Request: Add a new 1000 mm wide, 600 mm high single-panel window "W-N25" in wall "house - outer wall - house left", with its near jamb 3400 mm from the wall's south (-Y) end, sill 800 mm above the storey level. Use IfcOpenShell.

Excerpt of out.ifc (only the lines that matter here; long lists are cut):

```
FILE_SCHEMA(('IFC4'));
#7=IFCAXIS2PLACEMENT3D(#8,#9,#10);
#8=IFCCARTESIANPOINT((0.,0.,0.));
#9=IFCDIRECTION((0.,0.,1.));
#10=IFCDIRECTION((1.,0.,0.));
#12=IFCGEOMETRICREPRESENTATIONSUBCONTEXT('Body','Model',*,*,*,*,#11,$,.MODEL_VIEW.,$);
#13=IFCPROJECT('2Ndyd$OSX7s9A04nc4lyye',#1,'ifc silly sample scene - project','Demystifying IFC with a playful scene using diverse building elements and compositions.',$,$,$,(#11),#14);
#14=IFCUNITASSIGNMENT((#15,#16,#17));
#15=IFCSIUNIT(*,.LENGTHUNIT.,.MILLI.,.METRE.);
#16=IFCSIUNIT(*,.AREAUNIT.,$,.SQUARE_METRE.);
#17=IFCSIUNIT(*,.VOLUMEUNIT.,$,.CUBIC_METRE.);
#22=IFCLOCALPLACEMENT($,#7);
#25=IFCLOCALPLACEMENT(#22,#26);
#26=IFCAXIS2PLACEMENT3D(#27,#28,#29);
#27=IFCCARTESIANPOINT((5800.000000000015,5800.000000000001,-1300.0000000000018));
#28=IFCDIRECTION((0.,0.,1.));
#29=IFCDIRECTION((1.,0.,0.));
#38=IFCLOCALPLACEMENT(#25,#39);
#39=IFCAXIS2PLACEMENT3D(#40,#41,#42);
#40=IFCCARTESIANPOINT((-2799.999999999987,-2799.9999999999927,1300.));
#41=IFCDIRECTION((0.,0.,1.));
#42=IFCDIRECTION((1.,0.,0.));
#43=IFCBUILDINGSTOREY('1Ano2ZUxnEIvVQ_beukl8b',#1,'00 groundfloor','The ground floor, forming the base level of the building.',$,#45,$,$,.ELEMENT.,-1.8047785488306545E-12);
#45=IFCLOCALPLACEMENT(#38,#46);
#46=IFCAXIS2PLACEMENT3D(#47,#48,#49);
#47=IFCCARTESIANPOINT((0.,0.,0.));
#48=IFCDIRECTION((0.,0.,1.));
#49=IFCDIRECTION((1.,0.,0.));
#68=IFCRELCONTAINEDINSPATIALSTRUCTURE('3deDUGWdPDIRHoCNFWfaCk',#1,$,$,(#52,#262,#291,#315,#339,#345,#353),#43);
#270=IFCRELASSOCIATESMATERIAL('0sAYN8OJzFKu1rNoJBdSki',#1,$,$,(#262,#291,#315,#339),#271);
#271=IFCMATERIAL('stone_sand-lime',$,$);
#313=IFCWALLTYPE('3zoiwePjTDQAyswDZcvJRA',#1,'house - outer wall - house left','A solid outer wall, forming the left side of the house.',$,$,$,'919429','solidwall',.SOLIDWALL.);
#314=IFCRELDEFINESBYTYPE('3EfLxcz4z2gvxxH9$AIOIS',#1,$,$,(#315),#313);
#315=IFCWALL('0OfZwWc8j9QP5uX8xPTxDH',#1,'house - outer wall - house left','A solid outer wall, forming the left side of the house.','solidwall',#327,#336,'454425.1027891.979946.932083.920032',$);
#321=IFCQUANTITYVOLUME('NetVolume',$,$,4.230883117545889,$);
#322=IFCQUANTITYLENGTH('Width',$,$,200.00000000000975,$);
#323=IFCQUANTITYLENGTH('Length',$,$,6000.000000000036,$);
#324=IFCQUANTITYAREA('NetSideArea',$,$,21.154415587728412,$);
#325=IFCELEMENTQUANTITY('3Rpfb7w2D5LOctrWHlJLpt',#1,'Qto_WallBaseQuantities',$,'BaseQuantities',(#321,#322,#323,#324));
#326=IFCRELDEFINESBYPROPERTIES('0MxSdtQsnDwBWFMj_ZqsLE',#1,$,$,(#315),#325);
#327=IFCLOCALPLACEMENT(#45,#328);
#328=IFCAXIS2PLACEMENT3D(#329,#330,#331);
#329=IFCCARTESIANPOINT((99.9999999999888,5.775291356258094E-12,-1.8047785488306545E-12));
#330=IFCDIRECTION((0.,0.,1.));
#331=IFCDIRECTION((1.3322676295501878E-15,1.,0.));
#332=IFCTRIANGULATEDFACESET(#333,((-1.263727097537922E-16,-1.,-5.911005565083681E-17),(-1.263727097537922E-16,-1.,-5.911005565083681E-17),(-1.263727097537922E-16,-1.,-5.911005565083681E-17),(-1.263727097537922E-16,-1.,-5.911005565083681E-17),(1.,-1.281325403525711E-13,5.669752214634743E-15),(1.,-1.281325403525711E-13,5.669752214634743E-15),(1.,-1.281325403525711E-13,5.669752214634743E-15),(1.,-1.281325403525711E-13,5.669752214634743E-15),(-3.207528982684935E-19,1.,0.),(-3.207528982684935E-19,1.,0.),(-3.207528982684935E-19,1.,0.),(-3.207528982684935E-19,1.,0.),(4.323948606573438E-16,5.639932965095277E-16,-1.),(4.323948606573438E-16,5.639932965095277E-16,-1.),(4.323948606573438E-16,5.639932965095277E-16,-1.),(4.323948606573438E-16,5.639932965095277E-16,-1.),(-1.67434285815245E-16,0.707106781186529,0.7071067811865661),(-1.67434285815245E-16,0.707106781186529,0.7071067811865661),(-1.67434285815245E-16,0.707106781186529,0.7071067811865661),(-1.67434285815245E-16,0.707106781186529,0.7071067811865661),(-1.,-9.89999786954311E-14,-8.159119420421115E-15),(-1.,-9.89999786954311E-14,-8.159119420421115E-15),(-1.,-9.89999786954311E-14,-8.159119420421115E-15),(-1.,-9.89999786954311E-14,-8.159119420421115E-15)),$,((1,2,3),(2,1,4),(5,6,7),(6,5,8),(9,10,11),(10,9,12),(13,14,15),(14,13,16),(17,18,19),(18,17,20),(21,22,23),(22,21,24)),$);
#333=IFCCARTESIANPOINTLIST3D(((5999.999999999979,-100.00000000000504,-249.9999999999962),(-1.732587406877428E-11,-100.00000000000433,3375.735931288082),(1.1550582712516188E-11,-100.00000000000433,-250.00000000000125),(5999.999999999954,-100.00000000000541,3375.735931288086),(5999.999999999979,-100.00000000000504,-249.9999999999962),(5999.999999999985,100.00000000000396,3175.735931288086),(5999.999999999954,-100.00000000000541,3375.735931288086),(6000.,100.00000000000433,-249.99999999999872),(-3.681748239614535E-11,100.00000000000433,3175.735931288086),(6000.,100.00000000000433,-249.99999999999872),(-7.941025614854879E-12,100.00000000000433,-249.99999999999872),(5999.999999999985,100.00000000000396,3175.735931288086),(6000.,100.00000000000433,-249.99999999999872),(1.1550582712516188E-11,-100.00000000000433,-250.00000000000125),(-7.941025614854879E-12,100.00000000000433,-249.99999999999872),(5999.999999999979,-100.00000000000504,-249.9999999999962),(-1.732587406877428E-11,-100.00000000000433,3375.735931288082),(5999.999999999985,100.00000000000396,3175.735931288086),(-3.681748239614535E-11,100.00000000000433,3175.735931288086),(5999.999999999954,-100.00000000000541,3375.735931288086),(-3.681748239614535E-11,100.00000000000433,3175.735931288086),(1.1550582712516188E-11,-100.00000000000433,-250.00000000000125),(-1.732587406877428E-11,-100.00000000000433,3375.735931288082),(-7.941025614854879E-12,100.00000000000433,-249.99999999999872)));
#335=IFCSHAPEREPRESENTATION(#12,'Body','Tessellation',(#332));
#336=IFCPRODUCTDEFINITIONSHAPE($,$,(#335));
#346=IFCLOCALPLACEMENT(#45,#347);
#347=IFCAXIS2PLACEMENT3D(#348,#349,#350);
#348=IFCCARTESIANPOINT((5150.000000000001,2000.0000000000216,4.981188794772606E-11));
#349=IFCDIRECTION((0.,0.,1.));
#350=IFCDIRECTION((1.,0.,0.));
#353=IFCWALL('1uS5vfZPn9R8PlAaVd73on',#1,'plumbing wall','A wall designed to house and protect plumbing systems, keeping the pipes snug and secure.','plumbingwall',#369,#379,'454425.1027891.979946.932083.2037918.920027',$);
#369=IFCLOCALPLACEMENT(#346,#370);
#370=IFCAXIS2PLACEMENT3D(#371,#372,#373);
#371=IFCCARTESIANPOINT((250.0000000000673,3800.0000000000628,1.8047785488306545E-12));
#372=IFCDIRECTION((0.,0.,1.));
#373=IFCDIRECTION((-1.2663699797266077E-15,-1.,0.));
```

```python
import numpy as np
import ifcopenshell
import ifcopenshell.api.feature
import ifcopenshell.api.geometry
import ifcopenshell.api.pset
import ifcopenshell.api.root
import ifcopenshell.api.spatial
import ifcopenshell.geom
import ifcopenshell.util.element
import ifcopenshell.util.placement
import ifcopenshell.util.representation
import ifcopenshell.util.shape
import ifcopenshell.util.unit

model = ifcopenshell.open("out.ifc")
unit_scale = ifcopenshell.util.unit.calculate_unit_scale(model)
area_scale = ifcopenshell.util.unit.calculate_unit_scale(model, "AREAUNIT")
volume_scale = ifcopenshell.util.unit.calculate_unit_scale(model, "VOLUMEUNIT")
settings = ifcopenshell.geom.settings()


def volume(element):
    """Net volume in cubic metres, openings subtracted."""
    shape = ifcopenshell.geom.create_shape(settings, element)
    return ifcopenshell.util.shape.get_volume(shape.geometry)


wall = model.by_guid("0OfZwWc8j9QP5uX8xPTxDH")
storey = ifcopenshell.util.element.get_container(wall, ifc_class="IfcBuildingStorey")
context = ifcopenshell.util.representation.get_context(model, "Model", "Body", "MODEL_VIEW")
before = volume(wall)

width, height, from_end, sill = 1, 0.6, 3.4, 0.8  # metres

# The wall runs along its own X axis, and the end named is its -X end.
wall_shape = ifcopenshell.geom.create_shape(settings, wall)
x, y, z = ifcopenshell.util.shape.get_vertices(wall_shape.geometry).T
start = x.min() + from_end
face, thickness = float(y.min()), float(y.max() - y.min())
wall_matrix = ifcopenshell.util.placement.get_local_placement(wall.ObjectPlacement)
level = ifcopenshell.util.placement.get_local_placement(storey.ObjectPlacement)[2, 3]


def in_wall(x, y):
    """Placement at x, y metres in the wall's axes, at sill height."""
    matrix = wall_matrix.copy()
    matrix[:, 3] = wall_matrix @ np.array([x / unit_scale, y / unit_scale, 0.0, 1.0])
    matrix[2, 3] = level + sill / unit_scale
    return matrix


# Opening: a box that overshoots both wall faces by 50 mm.
opening = ifcopenshell.api.root.create_entity(model, ifc_class="IfcOpeningElement", predefined_type="OPENING")
box = ifcopenshell.api.geometry.add_wall_representation(
    model, context=context, length=width, height=height, thickness=thickness + 0.1
)
ifcopenshell.api.geometry.assign_representation(model, product=opening, representation=box)
ifcopenshell.api.geometry.edit_object_placement(model, product=opening, matrix=in_wall(start, face - 0.05), is_si=False)
ifcopenshell.api.feature.add_feature(model, feature=opening, element=wall)

window = ifcopenshell.api.root.create_entity(model, ifc_class="IfcWindow", name="W-N25", predefined_type="WINDOW")
window.OverallWidth, window.OverallHeight = width / unit_scale, height / unit_scale
window.PartitioningType = "SINGLE_PANEL"
body = ifcopenshell.api.geometry.add_window_representation(
    model,
    context=context,
    overall_width=window.OverallWidth,
    overall_height=window.OverallHeight,
    partition_type="SINGLE_PANEL",
)
ifcopenshell.api.geometry.assign_representation(model, product=window, representation=body)
ifcopenshell.api.spatial.assign_container(model, products=[window], relating_structure=storey)
ifcopenshell.api.feature.add_filling(model, opening=opening, element=window)

# Centre the window in the wall's thickness.
ifcopenshell.api.geometry.edit_object_placement(model, product=window, matrix=in_wall(start, face), is_si=False)
window_shape = ifcopenshell.geom.create_shape(settings, window)
depth = ifcopenshell.util.shape.get_vertices(window_shape.geometry)[:, 1]
offset = face + thickness / 2 - (depth.min() + depth.max()) / 2
ifcopenshell.api.geometry.edit_object_placement(model, product=window, matrix=in_wall(start, offset), is_si=False)

after = volume(wall)

# Update the wall's stored quantities.
qto = model.by_id(ifcopenshell.util.element.get_pset(wall, "Qto_WallBaseQuantities", should_inherit=False)["id"])
ifcopenshell.api.pset.edit_qto(model, qto=qto, properties={
    "NetVolume": after / volume_scale,
    "NetSideArea": after / thickness / area_scale,
})

print(f"wall volume {before:.3f} -> {after:.3f} m3")

model.write("out_edited.ifc")
```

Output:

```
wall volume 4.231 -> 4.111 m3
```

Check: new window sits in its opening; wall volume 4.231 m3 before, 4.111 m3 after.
